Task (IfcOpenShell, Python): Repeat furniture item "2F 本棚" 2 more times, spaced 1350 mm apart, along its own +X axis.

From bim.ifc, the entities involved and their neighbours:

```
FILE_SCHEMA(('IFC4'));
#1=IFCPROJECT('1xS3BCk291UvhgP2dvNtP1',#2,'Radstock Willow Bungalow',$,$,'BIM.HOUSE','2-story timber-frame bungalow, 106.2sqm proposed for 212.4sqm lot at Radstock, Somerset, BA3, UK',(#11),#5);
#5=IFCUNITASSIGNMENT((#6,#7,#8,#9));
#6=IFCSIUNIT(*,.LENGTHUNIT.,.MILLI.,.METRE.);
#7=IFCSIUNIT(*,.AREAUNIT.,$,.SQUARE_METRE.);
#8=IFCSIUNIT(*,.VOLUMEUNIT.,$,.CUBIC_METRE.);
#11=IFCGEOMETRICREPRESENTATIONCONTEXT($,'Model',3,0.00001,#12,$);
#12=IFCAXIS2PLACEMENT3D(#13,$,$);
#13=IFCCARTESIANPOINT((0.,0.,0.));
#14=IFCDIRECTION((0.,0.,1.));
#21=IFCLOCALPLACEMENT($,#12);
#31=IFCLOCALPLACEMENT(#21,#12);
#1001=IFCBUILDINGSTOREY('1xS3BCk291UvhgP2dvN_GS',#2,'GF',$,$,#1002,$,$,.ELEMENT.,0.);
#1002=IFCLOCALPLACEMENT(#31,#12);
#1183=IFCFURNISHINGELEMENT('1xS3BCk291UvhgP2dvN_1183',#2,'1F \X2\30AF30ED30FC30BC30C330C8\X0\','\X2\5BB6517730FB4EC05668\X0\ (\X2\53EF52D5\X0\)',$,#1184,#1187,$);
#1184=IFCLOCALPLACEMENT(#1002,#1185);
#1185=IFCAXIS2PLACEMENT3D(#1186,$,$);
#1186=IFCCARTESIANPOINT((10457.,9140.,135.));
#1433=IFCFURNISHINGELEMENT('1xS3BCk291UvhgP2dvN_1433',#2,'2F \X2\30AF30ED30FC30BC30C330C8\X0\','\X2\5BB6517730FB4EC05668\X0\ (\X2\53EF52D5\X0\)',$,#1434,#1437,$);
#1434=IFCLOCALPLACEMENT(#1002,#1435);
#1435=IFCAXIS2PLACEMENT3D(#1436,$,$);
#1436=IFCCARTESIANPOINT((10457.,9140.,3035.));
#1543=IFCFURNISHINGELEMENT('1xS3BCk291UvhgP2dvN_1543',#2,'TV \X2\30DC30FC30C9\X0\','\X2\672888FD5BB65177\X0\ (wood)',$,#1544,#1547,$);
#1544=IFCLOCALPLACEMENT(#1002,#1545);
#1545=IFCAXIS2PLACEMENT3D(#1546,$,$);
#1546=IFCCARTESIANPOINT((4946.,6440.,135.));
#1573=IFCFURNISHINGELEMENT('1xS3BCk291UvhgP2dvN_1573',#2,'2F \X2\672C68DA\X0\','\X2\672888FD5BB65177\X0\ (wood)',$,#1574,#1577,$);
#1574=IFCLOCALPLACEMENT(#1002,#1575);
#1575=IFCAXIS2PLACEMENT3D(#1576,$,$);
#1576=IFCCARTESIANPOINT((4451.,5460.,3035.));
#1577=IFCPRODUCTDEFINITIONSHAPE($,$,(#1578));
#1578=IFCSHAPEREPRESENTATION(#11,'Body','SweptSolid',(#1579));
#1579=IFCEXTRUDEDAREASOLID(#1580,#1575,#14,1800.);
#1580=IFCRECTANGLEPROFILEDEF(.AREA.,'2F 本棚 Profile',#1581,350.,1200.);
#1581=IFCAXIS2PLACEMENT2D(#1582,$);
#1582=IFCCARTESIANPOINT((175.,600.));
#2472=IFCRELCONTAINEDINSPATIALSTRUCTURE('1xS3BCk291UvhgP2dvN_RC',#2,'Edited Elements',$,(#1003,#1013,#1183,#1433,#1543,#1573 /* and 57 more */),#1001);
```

```python
import ifcopenshell
import ifcopenshell.api.geometry
import ifcopenshell.api.root
import ifcopenshell.util.element
import ifcopenshell.util.placement
import ifcopenshell.util.unit

model = ifcopenshell.open("bim.ifc")
unit_scale = ifcopenshell.util.unit.calculate_unit_scale(model)


def reuse_history(source, copy):
    """copy_class also copies each property set's owner history, people and application; keep the originals."""
    for rel in copy.IsDefinedBy:
        if rel.is_a("IfcRelDefinesByProperties") and (history := rel.RelatingPropertyDefinition.OwnerHistory):
            rel.RelatingPropertyDefinition.OwnerHistory = source.OwnerHistory
            ifcopenshell.util.element.remove_deep2(model, history)


source = model.by_id(1573)
base = ifcopenshell.util.placement.get_local_placement(source.ObjectPlacement)
step = base[:3, 0] * 1.35 / unit_scale

for i in range(1, 3):
    copy = ifcopenshell.api.root.copy_class(model, product=source)
    copy.Representation = ifcopenshell.util.element.copy_deep(
        model, source.Representation, exclude=["IfcGeometricRepresentationContext", "IfcRepresentationMap"]
    )
    reuse_history(source, copy)
    matrix = base.copy()
    matrix[:3, 3] += i * step
    print("added at", matrix[:3, 3].round(3) + 0.0)
    ifcopenshell.api.geometry.edit_object_placement(model, product=copy, matrix=matrix, is_si=False)

model.write("bim_v2.ifc")
```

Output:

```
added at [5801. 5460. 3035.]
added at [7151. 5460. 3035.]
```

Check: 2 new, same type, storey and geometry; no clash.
